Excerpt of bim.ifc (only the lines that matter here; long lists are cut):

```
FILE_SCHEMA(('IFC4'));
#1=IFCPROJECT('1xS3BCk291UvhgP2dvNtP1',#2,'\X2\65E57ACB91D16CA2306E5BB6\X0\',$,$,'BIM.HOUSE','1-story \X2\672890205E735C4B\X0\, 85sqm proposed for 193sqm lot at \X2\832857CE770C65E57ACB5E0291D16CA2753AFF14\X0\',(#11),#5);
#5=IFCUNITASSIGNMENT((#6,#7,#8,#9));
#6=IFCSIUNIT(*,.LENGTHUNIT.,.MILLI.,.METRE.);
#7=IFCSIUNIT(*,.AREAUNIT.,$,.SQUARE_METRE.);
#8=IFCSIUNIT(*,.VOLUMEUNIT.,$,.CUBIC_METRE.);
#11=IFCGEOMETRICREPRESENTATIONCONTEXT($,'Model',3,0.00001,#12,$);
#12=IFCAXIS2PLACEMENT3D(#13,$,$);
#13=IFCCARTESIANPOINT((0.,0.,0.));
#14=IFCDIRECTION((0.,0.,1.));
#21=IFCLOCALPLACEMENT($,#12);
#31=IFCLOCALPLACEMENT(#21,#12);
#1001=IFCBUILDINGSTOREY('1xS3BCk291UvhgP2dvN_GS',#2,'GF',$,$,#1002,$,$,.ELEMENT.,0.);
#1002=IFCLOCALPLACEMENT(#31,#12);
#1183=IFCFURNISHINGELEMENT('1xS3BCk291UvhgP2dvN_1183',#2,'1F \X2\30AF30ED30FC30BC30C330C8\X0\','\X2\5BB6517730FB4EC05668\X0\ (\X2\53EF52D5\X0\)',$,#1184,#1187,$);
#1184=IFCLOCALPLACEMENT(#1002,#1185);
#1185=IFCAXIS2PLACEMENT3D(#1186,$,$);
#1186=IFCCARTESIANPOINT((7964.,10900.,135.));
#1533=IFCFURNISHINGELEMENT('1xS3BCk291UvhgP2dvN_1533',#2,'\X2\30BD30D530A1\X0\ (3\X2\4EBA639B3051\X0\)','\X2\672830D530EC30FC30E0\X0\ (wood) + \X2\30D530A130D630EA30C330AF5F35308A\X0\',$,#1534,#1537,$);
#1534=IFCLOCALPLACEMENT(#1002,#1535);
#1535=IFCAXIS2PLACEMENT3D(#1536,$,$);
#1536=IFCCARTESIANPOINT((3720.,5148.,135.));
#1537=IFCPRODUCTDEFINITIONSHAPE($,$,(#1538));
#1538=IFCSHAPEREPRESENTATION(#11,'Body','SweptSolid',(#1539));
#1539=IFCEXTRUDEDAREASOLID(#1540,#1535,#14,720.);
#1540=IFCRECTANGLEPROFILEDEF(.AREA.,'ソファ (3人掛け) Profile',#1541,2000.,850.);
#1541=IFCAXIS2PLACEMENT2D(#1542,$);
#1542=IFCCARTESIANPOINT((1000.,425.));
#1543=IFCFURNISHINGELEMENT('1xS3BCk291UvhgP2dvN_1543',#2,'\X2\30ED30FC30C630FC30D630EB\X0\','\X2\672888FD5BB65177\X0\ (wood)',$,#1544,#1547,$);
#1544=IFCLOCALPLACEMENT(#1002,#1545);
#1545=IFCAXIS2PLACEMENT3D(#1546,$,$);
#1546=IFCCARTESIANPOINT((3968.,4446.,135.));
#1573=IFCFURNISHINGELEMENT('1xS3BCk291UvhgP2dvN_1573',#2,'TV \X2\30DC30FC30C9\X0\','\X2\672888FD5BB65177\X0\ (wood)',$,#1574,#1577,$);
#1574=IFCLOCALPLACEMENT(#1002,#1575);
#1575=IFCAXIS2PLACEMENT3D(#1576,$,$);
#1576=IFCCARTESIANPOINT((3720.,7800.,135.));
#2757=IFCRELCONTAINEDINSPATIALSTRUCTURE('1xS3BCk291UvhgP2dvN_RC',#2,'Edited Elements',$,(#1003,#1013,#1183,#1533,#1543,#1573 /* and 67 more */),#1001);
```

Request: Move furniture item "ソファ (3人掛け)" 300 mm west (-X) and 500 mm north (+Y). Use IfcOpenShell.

```python
import ifcopenshell
import ifcopenshell.api.geometry
import ifcopenshell.util.placement
import ifcopenshell.util.unit

model = ifcopenshell.open("bim.ifc")
unit_scale = ifcopenshell.util.unit.calculate_unit_scale(model)

item = model.by_id(1533)
matrix = ifcopenshell.util.placement.get_local_placement(item.ObjectPlacement)
matrix[0, 3] -= 0.3 / unit_scale
matrix[1, 3] += 0.5 / unit_scale
ifcopenshell.api.geometry.edit_object_placement(model, product=item, matrix=matrix, is_si=False)

print(ifcopenshell.util.placement.get_local_placement(item.ObjectPlacement).round(3) + 0.0)

model.write("bim_edited.ifc")
```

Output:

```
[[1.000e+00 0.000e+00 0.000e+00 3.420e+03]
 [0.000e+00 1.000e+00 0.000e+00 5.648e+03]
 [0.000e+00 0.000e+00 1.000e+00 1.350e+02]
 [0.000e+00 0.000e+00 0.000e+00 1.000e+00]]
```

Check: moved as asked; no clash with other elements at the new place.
